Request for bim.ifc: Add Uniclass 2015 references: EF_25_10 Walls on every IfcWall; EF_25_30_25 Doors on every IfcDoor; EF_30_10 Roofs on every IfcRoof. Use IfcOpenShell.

First a look at what the model holds.

```python
import ifcopenshell

model = ifcopenshell.open("bim.ifc")
print(model.schema)
print("classifications:", [c.Name for c in model.by_type("IfcClassification")])
for ifc_class in ("IfcDoor", "IfcRoof", "IfcStair", "IfcWall", "IfcWindow"):
    print(ifc_class, len(model.by_type(ifc_class)))
```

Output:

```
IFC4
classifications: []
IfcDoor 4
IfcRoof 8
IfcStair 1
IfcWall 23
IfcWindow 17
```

```python
import ifcopenshell
import ifcopenshell.api.classification

model = ifcopenshell.open("bim.ifc")

system = ifcopenshell.api.classification.add_classification(model, classification="Uniclass 2015")

codes = {
    "IfcWall": ("EF_25_10", "Walls"),
    "IfcDoor": ("EF_25_30_25", "Doors"),
    "IfcRoof": ("EF_30_10", "Roofs"),
}
for ifc_class, (code, name) in codes.items():
    products = model.by_type(ifc_class)
    ifcopenshell.api.classification.add_reference(
        model, products=products, classification=system, identification=code, name=name
    )
    print(code, len(products))

model.write("bim_v2.ifc")
```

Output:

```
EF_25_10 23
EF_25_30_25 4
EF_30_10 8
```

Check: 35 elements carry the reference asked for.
